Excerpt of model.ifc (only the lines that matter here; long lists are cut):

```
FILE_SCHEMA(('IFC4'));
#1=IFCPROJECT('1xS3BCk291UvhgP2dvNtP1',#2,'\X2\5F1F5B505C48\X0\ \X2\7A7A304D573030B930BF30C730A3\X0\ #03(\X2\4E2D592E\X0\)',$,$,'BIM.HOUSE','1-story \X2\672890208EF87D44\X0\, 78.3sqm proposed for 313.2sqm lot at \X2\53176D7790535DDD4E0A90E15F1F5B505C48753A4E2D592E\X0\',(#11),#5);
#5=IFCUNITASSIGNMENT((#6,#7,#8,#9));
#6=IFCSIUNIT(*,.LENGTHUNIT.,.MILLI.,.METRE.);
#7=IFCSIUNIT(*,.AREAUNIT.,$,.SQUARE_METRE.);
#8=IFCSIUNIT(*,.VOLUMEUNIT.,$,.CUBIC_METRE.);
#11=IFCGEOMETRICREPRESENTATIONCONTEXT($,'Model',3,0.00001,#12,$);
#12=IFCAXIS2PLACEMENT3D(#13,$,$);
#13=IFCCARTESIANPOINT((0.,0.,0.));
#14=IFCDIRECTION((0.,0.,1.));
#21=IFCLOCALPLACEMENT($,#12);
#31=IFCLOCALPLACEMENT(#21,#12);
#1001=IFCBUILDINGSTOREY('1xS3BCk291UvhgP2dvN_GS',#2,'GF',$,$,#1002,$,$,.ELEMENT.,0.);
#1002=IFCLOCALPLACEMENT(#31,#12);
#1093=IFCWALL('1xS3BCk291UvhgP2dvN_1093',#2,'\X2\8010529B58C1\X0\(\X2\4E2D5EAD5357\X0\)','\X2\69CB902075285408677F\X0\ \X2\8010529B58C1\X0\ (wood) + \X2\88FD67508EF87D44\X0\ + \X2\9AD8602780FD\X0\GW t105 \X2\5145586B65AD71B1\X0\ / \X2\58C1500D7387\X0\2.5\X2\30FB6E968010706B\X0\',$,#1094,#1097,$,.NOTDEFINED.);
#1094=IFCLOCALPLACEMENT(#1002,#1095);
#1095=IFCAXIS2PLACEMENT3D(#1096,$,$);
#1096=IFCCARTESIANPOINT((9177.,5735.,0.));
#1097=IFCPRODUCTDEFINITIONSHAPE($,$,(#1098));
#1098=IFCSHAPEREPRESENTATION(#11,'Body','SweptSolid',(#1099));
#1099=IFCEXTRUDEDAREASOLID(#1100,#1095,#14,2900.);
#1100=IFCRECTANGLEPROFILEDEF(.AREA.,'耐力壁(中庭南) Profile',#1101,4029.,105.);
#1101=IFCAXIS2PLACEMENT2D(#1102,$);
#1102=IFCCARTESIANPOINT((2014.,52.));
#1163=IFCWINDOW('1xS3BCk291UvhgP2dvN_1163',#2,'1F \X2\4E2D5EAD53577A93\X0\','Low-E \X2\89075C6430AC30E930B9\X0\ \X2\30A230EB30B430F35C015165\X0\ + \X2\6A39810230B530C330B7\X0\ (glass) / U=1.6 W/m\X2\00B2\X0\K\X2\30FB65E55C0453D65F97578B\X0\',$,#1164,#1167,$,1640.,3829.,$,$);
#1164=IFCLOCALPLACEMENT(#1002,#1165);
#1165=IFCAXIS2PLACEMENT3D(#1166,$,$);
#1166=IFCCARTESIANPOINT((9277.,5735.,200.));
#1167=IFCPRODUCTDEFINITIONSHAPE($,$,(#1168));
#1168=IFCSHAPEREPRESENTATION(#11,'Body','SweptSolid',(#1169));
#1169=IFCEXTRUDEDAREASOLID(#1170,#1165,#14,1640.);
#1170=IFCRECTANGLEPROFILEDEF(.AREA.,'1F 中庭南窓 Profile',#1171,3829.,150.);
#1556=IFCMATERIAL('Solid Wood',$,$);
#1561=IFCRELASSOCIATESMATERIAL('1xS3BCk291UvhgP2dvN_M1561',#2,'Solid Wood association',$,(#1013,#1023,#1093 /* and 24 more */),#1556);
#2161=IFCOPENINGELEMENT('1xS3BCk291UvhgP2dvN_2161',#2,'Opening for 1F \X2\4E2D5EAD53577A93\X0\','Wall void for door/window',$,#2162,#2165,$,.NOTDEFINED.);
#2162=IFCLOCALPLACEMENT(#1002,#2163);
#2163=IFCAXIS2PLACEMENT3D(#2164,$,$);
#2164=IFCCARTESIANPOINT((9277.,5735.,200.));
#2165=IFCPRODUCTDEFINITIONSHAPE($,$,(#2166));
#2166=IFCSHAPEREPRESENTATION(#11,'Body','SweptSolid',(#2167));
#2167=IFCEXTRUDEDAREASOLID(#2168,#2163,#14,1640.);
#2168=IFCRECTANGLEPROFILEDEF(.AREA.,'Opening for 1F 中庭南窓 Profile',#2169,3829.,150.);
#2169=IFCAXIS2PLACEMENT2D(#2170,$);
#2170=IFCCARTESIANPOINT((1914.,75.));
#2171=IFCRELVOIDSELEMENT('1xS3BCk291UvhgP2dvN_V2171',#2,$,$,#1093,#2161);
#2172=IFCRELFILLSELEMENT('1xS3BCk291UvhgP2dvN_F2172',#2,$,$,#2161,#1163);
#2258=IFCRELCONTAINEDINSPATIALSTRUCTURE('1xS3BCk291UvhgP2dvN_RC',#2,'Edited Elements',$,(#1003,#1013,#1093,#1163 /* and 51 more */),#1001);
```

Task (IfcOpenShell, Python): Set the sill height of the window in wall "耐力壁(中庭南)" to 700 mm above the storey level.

```python
import numpy as np
import ifcopenshell
import ifcopenshell.api.geometry
import ifcopenshell.geom
import ifcopenshell.util.element
import ifcopenshell.util.placement
import ifcopenshell.util.shape
import ifcopenshell.util.unit

model = ifcopenshell.open("model.ifc")
unit_scale = ifcopenshell.util.unit.calculate_unit_scale(model)

window = model.by_guid("1xS3BCk291UvhgP2dvN_1163")
opening = window.FillsVoids[0].RelatingOpeningElement
storey = ifcopenshell.util.element.get_container(window, ifc_class="IfcBuildingStorey")
level = ifcopenshell.util.placement.get_local_placement(storey.ObjectPlacement)[2, 3]

# The opening's origin need not be at the sill, so measure its lowest point.
shape = ifcopenshell.geom.create_shape(ifcopenshell.geom.settings(), opening)
bottom = ifcopenshell.util.shape.get_shape_bottom_elevation(shape, shape.geometry) / unit_scale
dz = level + 700.0 - bottom

shift = np.array([0.0, 0.0, dz])
# The window is not placed relative to its opening, so move both.
for product in (opening, window):
    matrix = ifcopenshell.util.placement.get_local_placement(product.ObjectPlacement)
    matrix[:3, 3] += shift
    ifcopenshell.api.geometry.edit_object_placement(model, product=product, matrix=matrix, is_si=False)

print(f"moved by {dz * unit_scale:+.3f} m")

model.write("model-out.ifc")
```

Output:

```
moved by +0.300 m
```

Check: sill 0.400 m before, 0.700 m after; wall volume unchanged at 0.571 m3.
